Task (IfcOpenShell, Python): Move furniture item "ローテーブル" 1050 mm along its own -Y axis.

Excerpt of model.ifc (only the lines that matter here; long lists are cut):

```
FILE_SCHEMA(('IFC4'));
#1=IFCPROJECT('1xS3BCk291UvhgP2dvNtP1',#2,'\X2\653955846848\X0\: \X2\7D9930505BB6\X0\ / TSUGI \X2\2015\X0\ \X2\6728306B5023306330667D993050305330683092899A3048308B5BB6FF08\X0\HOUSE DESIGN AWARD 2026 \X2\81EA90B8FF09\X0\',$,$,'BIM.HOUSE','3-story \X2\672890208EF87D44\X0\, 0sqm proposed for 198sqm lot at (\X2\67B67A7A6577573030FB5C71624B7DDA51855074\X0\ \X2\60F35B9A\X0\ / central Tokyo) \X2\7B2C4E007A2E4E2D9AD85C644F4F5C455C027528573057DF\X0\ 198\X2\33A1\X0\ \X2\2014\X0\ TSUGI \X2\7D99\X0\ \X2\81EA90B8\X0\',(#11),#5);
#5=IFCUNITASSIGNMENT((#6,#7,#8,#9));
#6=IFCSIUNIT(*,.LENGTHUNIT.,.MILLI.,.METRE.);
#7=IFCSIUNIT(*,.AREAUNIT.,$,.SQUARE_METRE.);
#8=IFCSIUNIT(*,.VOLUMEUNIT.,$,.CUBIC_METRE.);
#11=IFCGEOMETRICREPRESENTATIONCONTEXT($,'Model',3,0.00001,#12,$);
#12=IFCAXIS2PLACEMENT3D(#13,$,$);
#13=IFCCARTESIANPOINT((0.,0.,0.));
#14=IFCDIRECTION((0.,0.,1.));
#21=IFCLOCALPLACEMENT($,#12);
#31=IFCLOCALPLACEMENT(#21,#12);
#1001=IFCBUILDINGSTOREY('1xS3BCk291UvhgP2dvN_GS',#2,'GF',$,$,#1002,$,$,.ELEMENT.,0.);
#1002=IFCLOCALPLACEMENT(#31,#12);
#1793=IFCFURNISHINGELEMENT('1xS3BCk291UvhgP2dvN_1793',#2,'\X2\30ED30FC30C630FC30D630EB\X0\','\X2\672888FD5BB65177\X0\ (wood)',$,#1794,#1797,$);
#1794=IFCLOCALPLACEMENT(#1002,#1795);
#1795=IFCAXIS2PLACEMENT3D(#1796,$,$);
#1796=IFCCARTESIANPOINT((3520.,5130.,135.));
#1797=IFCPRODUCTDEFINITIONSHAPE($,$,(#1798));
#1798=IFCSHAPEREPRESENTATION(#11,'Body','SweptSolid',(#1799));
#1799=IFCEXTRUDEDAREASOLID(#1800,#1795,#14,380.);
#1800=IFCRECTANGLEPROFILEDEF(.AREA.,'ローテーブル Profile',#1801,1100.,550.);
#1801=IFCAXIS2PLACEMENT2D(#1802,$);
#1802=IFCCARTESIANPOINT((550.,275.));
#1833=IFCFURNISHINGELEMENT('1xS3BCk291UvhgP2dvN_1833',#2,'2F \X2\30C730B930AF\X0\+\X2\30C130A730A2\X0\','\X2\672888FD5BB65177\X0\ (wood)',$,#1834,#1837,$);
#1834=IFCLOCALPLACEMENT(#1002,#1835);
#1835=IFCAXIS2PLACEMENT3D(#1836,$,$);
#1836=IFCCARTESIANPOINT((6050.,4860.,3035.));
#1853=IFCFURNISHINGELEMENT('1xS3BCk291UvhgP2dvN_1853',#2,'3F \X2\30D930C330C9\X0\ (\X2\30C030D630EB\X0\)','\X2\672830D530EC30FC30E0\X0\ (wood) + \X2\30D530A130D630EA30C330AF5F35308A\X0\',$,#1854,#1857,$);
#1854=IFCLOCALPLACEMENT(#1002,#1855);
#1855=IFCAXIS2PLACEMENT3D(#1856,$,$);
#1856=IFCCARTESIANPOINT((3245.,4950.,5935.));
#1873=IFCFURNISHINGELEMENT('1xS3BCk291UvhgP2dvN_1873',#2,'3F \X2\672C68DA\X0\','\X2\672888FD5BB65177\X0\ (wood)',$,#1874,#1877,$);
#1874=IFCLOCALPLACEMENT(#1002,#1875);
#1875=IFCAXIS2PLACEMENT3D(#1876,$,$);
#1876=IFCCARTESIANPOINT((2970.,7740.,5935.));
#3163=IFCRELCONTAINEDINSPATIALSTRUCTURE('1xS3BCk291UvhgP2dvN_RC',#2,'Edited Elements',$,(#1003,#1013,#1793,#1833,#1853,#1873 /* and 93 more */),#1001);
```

```python
import ifcopenshell
import ifcopenshell.api.geometry
import ifcopenshell.util.placement
import ifcopenshell.util.unit

model = ifcopenshell.open("model.ifc")
unit_scale = ifcopenshell.util.unit.calculate_unit_scale(model)

item = model.by_guid("1xS3BCk291UvhgP2dvN_1793")
matrix = ifcopenshell.util.placement.get_local_placement(item.ObjectPlacement)
matrix[:3, 3] -= matrix[:3, 1] * 1.05 / unit_scale
ifcopenshell.api.geometry.edit_object_placement(model, product=item, matrix=matrix, is_si=False)

print(ifcopenshell.util.placement.get_local_placement(item.ObjectPlacement).round(3) + 0.0)

model.write("model_rev.ifc")
```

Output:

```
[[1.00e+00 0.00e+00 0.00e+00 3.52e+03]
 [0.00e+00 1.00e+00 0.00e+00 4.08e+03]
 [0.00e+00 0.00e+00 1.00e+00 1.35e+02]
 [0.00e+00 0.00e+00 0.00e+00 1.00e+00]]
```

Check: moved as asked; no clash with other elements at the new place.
